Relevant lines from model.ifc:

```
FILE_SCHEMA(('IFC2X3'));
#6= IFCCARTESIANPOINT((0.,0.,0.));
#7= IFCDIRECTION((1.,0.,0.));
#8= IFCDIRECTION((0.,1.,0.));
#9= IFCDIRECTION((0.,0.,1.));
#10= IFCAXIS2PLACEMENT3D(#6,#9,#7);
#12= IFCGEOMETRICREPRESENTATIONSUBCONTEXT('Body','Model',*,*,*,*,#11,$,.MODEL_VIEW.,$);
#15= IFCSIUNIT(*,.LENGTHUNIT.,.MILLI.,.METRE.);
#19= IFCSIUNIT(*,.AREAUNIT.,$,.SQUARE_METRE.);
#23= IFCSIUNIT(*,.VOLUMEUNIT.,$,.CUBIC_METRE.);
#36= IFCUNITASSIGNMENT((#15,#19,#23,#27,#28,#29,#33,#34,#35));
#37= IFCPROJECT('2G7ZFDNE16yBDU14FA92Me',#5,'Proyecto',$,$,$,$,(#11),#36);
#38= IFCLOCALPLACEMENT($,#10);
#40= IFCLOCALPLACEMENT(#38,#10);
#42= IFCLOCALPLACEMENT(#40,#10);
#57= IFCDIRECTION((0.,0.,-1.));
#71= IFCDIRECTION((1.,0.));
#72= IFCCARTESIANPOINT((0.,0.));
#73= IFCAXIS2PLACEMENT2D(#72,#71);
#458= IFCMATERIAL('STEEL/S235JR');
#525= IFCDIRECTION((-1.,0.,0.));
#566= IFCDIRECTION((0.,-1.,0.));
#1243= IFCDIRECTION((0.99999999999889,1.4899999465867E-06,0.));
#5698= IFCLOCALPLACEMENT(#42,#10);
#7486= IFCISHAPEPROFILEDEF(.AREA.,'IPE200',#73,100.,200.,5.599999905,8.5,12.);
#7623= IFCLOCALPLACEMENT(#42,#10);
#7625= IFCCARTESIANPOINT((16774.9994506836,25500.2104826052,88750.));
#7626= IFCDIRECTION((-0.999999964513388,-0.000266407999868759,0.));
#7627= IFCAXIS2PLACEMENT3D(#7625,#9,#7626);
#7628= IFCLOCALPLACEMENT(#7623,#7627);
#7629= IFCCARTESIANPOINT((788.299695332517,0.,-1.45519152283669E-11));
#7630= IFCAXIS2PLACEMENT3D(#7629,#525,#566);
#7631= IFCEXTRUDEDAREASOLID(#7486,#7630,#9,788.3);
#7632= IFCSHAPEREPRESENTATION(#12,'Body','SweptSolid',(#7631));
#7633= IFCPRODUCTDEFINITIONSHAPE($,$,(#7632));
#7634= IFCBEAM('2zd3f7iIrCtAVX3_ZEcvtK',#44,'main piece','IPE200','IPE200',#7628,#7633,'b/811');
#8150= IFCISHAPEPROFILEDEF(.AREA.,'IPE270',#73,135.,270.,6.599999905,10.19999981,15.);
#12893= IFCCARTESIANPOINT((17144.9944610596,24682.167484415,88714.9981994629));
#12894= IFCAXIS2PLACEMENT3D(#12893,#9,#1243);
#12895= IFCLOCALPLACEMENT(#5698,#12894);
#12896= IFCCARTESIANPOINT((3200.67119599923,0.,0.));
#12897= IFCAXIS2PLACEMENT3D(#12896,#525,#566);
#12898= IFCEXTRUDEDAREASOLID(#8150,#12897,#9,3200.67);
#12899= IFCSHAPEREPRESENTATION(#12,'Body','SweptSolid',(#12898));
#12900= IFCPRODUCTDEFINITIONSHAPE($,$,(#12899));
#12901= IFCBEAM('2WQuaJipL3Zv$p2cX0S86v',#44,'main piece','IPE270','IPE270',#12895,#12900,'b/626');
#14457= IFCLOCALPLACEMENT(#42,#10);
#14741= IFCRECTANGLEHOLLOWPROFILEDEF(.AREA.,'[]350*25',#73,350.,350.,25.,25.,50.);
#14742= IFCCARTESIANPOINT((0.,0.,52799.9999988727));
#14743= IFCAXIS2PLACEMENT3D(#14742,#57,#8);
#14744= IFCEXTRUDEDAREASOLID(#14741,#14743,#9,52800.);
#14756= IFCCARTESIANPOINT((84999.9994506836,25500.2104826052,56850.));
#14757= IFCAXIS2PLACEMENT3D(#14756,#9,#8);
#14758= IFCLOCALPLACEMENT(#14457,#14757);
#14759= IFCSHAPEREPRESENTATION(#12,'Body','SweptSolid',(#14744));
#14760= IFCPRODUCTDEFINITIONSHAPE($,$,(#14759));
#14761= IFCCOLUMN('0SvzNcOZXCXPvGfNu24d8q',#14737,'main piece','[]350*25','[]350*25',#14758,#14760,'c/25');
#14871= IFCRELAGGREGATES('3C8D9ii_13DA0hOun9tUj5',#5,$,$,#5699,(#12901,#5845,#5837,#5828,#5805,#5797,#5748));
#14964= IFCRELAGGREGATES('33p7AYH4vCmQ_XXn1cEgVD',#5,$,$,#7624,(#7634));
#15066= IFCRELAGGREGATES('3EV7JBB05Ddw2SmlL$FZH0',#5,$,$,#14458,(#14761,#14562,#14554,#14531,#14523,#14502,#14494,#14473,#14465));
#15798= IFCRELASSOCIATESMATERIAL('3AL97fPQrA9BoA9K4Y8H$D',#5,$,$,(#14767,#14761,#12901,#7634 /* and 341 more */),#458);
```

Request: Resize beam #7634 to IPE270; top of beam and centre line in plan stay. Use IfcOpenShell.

```python
import ifcopenshell
import ifcopenshell.util.element
import ifcopenshell.util.representation

model = ifcopenshell.open("model.ifc")

member = model.by_id(7634)
source = next(p for p in model.by_type("IfcIShapeProfileDef") if p.ProfileName == "IPE270")

body = ifcopenshell.util.representation.get_representation(member, "Model", "Body")
solid = body.Items[0]
old_profile = solid.SweptArea

# Copy the section's sizes but keep this member's own profile position.
profile = ifcopenshell.util.element.copy(model, source)
# Profiles are centred, so shift by half the change in depth to hold the top.
shift = (old_profile.OverallDepth - profile.OverallDepth) / 2
x, y = old_profile.Position.Location.Coordinates
up = (0.0, 1.0)  # upwards, in the solid's own plane
location = model.createIfcCartesianPoint((x + up[0] * shift, y + up[1] * shift))
profile.Position = model.createIfcAxis2Placement2D(location, old_profile.Position.RefDirection)
solid.SweptArea = profile
if not model.get_total_inverses(old_profile):
    ifcopenshell.util.element.remove_deep2(model, old_profile)
member.Description = member.Description.replace("IPE200", "IPE270")
member.ObjectType = member.ObjectType.replace("IPE200", "IPE270")

print(solid.SweptArea)

model.write("model_edited.ifc")
```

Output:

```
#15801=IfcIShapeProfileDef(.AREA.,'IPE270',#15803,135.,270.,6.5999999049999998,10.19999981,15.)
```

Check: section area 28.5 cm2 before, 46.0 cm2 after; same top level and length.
